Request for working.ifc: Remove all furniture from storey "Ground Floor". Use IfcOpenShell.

First a look at what the model holds.

```python
import ifcopenshell
import ifcopenshell.util.element

model = ifcopenshell.open("working.ifc")
print(model.schema)
storey = next(s for s in model.by_type("IfcBuildingStorey") if s.Name == "Ground Floor")
furniture = [e for e in ifcopenshell.util.element.get_decomposition(storey) if e.is_a("IfcFurnishingElement")]
seen = {}
for e in furniture:
    element_type = ifcopenshell.util.element.get_type(e)
    name = element_type.Name if element_type not in (None, e) else None
    seen[name] = seen.get(name, 0) + 1
for name, count in sorted(seen.items(), key=str):
    print(count, "x", name)
```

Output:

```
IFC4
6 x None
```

```python
import ifcopenshell
import ifcopenshell.api.root
import ifcopenshell.util.element

model = ifcopenshell.open("working.ifc")

storey = next(s for s in model.by_type("IfcBuildingStorey") if s.Name == "Ground Floor")
furniture = [e for e in ifcopenshell.util.element.get_decomposition(storey) if e.is_a("IfcFurnishingElement")]

for e in furniture:
    ifcopenshell.api.root.remove_product(model, product=e)
print(len(furniture), "removed")

model.write("working_rev.ifc")
```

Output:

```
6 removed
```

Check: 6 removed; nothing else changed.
